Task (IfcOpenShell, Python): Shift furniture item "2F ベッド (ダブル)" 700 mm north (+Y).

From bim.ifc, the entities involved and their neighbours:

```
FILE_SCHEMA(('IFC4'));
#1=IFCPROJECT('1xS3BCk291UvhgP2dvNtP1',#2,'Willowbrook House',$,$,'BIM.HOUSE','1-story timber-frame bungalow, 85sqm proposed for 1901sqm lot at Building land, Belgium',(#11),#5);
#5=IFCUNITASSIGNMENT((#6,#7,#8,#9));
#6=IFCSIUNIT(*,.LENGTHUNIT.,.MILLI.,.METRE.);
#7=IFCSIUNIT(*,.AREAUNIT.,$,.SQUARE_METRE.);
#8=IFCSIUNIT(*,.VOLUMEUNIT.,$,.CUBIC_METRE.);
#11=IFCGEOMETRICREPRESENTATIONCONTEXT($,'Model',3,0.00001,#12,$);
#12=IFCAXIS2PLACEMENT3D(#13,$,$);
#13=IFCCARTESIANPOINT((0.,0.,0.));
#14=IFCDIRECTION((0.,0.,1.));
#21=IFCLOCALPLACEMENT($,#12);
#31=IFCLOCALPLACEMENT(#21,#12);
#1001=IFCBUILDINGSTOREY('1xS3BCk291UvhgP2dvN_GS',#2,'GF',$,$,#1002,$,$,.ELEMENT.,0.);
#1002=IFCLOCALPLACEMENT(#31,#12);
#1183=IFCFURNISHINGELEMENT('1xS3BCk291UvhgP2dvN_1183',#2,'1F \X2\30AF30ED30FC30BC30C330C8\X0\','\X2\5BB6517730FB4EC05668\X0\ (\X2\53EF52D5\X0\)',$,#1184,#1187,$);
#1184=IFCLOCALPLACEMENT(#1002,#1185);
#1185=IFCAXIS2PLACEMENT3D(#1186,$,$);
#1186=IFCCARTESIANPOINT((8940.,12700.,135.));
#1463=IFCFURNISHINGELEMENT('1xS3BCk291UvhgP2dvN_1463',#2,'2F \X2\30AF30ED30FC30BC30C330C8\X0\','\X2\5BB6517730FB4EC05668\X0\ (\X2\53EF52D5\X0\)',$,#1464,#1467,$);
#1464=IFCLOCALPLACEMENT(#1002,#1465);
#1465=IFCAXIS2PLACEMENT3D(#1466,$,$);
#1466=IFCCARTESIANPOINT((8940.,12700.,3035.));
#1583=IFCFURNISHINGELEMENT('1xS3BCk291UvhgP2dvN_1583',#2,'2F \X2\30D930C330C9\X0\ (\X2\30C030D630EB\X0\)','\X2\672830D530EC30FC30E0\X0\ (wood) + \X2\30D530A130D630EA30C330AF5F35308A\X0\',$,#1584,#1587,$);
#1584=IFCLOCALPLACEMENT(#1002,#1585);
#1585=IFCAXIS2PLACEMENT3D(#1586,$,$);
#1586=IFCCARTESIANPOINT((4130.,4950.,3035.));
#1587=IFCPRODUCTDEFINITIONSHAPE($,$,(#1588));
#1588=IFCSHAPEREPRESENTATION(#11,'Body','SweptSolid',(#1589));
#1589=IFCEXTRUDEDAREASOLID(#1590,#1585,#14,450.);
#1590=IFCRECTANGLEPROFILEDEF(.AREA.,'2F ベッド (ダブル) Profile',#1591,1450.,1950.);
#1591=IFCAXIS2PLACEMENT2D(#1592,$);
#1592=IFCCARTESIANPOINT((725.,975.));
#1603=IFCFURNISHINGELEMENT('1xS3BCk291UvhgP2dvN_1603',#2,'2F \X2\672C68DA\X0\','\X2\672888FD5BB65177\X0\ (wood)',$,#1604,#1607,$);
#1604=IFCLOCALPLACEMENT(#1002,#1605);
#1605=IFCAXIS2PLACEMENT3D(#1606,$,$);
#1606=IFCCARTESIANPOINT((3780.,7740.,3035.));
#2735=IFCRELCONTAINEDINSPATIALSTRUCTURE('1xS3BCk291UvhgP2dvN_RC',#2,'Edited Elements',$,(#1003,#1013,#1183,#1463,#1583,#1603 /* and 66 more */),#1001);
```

```python
import ifcopenshell
import ifcopenshell.api.geometry
import ifcopenshell.util.placement

model = ifcopenshell.open("bim.ifc")

item = model.by_guid("1xS3BCk291UvhgP2dvN_1583")
matrix = ifcopenshell.util.placement.get_local_placement(item.ObjectPlacement)
matrix[1, 3] += 700.0
ifcopenshell.api.geometry.edit_object_placement(model, product=item, matrix=matrix, is_si=False)

print(ifcopenshell.util.placement.get_local_placement(item.ObjectPlacement).round(3) + 0.0)

model.write("bim_v2.ifc")
```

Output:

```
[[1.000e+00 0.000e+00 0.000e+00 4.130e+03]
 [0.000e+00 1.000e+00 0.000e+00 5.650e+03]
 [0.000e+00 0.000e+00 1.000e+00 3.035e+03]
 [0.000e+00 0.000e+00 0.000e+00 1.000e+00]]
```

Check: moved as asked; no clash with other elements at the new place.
